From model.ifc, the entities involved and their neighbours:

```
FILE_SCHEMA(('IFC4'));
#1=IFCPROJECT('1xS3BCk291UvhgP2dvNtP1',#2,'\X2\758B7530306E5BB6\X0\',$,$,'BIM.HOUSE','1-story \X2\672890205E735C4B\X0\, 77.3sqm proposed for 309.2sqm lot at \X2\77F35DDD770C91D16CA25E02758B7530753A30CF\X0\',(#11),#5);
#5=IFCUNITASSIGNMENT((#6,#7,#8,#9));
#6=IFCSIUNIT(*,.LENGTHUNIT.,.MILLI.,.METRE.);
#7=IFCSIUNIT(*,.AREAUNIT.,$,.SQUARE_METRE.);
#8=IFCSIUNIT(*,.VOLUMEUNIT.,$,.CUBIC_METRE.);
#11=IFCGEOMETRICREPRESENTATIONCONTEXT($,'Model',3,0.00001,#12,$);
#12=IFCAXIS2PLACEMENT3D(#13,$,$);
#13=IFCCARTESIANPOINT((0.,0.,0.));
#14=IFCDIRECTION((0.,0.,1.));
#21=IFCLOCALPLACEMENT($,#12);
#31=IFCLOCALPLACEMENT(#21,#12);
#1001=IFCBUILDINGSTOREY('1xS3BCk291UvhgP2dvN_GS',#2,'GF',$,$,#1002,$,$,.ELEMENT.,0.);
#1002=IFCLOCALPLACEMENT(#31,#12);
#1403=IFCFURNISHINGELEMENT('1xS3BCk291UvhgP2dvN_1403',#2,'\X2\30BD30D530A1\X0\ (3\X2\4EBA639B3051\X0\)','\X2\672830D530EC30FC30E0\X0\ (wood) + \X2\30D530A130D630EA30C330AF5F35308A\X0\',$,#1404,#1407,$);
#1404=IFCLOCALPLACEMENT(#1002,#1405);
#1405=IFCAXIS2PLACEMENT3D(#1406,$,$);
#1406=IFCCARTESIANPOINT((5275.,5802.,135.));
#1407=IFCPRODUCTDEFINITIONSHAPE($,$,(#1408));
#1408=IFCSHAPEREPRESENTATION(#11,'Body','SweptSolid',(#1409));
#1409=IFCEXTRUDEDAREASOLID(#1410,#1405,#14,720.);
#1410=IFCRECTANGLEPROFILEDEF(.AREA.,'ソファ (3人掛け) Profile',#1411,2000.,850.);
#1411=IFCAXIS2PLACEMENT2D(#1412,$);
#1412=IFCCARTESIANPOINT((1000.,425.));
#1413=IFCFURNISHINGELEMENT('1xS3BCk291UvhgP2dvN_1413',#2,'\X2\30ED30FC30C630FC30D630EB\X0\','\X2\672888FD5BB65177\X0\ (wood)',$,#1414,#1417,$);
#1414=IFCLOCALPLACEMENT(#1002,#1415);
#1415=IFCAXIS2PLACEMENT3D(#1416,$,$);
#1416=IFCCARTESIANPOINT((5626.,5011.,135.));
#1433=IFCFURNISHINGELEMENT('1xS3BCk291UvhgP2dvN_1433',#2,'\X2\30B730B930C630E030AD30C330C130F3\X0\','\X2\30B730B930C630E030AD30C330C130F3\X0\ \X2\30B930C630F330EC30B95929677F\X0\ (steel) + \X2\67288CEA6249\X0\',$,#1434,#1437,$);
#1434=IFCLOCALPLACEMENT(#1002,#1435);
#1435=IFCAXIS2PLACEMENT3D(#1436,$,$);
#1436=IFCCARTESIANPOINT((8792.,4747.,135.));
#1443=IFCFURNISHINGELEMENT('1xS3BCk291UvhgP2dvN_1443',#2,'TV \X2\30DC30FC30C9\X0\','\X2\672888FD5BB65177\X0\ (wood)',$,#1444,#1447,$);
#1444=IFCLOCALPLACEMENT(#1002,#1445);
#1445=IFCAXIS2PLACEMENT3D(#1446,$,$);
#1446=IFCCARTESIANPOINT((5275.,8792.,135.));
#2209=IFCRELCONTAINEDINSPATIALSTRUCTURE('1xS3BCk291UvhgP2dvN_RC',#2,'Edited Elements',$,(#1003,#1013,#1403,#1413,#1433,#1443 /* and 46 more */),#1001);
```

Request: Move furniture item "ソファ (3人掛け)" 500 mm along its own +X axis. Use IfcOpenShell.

```python
import ifcopenshell
import ifcopenshell.api.geometry
import ifcopenshell.util.placement
import ifcopenshell.util.unit

model = ifcopenshell.open("model.ifc")
unit_scale = ifcopenshell.util.unit.calculate_unit_scale(model)

item = model.by_guid("1xS3BCk291UvhgP2dvN_1403")
matrix = ifcopenshell.util.placement.get_local_placement(item.ObjectPlacement)
matrix[:3, 3] += matrix[:3, 0] * 0.5 / unit_scale
ifcopenshell.api.geometry.edit_object_placement(model, product=item, matrix=matrix, is_si=False)

print(ifcopenshell.util.placement.get_local_placement(item.ObjectPlacement).round(3) + 0.0)

model.write("model_updated.ifc")
```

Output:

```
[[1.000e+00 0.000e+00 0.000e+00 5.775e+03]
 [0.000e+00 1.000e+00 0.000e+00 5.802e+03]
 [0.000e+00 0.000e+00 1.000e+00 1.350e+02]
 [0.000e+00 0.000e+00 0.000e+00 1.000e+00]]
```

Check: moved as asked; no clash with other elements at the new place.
